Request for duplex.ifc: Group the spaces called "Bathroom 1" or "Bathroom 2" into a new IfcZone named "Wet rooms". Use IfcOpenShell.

First a look at what the model holds.

```python
import ifcopenshell

model = ifcopenshell.open("duplex.ifc")
print(model.schema)
seen = {}
for space in model.by_type("IfcSpace"):
    seen[space.LongName] = seen.get(space.LongName, 0) + 1
for name, count in sorted(seen.items(), key=str):
    print(count, "x", name)
print("zones:", [z.Name for z in model.by_type("IfcZone")][:20])
```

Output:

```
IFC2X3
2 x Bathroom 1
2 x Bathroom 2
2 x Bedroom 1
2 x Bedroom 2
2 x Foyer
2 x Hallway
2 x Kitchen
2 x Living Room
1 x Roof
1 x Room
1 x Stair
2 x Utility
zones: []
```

```python
import ifcopenshell
import ifcopenshell.api.group
import ifcopenshell.api.root

model = ifcopenshell.open("duplex.ifc")

names = {"Bathroom 1", "Bathroom 2"}
spaces = [s for s in model.by_type("IfcSpace") if s.LongName in names]

zone = ifcopenshell.api.root.create_entity(model, ifc_class="IfcZone", name="Wet rooms")
ifcopenshell.api.group.assign_group(model, products=spaces, group=zone)
print(len(spaces), "spaces in", zone.Name)

model.write("duplex_edited.ifc")
```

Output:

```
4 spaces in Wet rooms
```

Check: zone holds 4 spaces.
